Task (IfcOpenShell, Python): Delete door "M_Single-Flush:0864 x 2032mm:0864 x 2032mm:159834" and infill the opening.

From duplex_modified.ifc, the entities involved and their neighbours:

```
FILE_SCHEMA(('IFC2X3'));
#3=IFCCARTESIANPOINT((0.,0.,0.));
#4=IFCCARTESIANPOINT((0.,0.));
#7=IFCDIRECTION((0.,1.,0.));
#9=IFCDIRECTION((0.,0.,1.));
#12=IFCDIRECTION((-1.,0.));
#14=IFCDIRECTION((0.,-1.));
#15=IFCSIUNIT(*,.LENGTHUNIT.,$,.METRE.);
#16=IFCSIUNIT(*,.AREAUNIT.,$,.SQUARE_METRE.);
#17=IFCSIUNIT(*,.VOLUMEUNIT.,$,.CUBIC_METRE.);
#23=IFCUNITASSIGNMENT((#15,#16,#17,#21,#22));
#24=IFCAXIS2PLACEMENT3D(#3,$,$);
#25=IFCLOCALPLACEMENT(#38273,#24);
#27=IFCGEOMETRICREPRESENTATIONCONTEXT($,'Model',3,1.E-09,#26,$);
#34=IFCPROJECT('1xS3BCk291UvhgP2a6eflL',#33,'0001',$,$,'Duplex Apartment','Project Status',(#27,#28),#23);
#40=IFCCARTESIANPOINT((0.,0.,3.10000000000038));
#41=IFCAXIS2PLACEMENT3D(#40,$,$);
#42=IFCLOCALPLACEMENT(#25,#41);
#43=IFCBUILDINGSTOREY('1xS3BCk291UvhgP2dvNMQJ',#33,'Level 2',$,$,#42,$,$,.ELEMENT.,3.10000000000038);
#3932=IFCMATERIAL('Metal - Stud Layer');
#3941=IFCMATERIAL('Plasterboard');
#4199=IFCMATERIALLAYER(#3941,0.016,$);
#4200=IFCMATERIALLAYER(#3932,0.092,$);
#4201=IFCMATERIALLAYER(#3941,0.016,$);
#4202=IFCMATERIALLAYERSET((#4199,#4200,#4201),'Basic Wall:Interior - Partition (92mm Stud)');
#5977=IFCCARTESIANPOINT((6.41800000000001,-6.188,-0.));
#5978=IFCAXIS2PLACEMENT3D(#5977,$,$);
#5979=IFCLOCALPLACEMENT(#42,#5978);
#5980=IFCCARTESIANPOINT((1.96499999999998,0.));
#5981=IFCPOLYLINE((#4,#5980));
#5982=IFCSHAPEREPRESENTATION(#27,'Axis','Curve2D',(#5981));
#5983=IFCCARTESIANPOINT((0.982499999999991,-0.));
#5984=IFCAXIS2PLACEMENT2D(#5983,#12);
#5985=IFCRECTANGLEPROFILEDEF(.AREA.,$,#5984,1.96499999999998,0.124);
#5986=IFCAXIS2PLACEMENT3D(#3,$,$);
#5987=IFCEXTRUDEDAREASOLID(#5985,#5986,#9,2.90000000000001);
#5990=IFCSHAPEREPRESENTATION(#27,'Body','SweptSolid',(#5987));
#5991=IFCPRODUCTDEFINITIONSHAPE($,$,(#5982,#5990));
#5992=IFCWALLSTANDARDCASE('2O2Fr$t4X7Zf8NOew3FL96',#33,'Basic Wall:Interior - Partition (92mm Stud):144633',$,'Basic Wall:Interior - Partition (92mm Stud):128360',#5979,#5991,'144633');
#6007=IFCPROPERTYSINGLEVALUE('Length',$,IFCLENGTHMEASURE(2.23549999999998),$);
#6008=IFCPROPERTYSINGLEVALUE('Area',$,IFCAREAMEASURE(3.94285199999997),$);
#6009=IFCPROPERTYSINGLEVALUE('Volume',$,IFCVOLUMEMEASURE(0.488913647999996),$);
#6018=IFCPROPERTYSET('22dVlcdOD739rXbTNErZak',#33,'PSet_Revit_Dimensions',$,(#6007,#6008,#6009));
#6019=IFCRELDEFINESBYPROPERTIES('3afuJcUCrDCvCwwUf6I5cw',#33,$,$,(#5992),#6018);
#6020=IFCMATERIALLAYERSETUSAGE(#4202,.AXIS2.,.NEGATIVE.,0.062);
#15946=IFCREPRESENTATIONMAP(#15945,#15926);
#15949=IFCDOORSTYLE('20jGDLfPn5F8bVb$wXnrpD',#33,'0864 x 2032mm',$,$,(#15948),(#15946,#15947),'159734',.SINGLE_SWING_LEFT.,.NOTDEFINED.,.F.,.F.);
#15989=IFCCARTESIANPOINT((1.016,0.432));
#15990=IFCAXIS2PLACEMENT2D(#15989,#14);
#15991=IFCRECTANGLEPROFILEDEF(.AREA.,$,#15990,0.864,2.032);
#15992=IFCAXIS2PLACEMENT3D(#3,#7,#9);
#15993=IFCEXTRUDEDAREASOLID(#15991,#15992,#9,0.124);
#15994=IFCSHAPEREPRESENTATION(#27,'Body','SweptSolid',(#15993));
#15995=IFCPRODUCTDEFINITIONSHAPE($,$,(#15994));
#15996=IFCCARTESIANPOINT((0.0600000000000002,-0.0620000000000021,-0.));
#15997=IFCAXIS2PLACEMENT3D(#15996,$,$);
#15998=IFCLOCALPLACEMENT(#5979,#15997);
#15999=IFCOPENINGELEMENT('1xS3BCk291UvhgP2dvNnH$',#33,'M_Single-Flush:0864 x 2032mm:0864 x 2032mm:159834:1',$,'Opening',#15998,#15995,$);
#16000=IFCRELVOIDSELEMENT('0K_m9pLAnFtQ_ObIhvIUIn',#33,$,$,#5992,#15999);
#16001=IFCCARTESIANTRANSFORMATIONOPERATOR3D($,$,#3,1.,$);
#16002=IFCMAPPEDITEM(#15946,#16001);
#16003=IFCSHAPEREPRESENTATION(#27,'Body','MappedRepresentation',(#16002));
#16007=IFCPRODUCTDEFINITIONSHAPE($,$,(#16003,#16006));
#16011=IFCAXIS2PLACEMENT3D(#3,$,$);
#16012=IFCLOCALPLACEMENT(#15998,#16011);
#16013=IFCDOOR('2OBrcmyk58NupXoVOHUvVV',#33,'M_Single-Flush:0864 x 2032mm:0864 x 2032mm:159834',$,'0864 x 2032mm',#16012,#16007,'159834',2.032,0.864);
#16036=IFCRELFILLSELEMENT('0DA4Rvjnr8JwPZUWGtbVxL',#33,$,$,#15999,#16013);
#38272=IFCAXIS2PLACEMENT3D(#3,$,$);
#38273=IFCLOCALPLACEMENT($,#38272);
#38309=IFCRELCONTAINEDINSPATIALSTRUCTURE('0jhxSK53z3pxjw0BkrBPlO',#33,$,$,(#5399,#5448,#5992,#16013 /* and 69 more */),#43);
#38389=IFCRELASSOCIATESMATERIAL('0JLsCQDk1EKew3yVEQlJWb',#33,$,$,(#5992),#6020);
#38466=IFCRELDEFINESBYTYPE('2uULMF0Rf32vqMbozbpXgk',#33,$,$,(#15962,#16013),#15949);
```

```python
import ifcopenshell
import ifcopenshell.api.feature
import ifcopenshell.api.pset
import ifcopenshell.api.root
import ifcopenshell.geom
import ifcopenshell.util.element
import ifcopenshell.util.shape
import ifcopenshell.util.unit

model = ifcopenshell.open("duplex_modified.ifc")
area_scale = ifcopenshell.util.unit.calculate_unit_scale(model, "AREAUNIT")
volume_scale = ifcopenshell.util.unit.calculate_unit_scale(model, "VOLUMEUNIT")
settings = ifcopenshell.geom.settings()


def volume(element):
    """Net volume in cubic metres, openings subtracted."""
    shape = ifcopenshell.geom.create_shape(settings, element)
    return ifcopenshell.util.shape.get_volume(shape.geometry)


door = model.by_guid("2OBrcmyk58NupXoVOHUvVV")
opening = door.FillsVoids[0].RelatingOpeningElement
wall = opening.VoidsElements[0].RelatingBuildingElement
before = volume(wall)

ifcopenshell.api.root.remove_product(model, product=door)
ifcopenshell.api.feature.remove_feature(model, feature=opening)

after = volume(wall)
thickness = 0.124  # wall thickness in metres

# Update the wall's stored quantities.
pset = model.by_id(ifcopenshell.util.element.get_pset(wall, "PSet_Revit_Dimensions", should_inherit=False)["id"])
ifcopenshell.api.pset.edit_pset(model, pset=pset, properties={
    "Area": model.create_entity("IfcAreaMeasure", after / thickness / area_scale),
    "Volume": model.create_entity("IfcVolumeMeasure", after / volume_scale),
})

print(f"wall volume {before:.3f} -> {after:.3f} m3")

model.write("duplex_modified_updated.ifc")
```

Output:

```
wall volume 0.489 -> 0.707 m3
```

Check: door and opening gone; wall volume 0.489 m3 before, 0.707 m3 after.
